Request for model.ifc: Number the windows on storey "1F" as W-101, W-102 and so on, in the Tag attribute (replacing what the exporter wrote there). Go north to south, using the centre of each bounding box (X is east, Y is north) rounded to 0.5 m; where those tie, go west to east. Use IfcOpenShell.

First a look at what the model holds.

```python
import ifcopenshell
import ifcopenshell.util.element
import ifcopenshell.util.placement

model = ifcopenshell.open("model.ifc")
print(model.schema)
storey = next(s for s in model.by_type("IfcBuildingStorey") if s.Name == "1F")
windows = [e for e in ifcopenshell.util.element.get_decomposition(storey) if e.is_a("IfcWindow")]
for e in sorted(windows, key=lambda e: e.id()):
    origin = ifcopenshell.util.placement.get_local_placement(e.ObjectPlacement)[:3, 3]
    print(e.id(), e.Tag, e.Name, origin.round(2) + 0.0, sep=" | ")
```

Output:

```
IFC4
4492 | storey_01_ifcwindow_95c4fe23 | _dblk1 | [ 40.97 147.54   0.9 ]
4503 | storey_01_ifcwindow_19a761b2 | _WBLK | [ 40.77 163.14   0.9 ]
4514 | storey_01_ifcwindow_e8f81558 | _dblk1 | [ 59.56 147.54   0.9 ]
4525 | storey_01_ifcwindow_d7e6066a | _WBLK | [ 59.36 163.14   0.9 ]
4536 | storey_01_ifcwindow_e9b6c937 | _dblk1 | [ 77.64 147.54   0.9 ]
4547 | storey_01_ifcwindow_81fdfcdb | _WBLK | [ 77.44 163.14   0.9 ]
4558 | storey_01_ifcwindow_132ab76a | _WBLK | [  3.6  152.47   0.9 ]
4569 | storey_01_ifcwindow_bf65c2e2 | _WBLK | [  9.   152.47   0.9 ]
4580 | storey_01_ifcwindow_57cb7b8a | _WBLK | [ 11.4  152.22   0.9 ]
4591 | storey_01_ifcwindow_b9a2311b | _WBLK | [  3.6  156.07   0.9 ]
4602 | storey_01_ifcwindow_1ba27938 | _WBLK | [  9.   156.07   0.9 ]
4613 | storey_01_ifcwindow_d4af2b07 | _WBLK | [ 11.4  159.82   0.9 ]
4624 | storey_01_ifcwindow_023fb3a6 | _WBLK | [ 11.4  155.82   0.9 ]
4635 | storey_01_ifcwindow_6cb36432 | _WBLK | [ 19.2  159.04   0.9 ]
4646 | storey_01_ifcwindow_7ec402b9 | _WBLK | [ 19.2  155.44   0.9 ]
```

```python
import ifcopenshell
import ifcopenshell.geom
import ifcopenshell.util.element
import ifcopenshell.util.shape

model = ifcopenshell.open("model.ifc")
settings = ifcopenshell.geom.settings()
settings.set("use-world-coords", True)


def centre(element):
    shape = ifcopenshell.geom.create_shape(settings, element)
    return ifcopenshell.util.shape.get_bbox_centroid(shape.geometry)


storey = next(s for s in model.by_type("IfcBuildingStorey") if s.Name == "1F")
windows = [e for e in ifcopenshell.util.element.get_decomposition(storey) if e.is_a("IfcWindow")]

# Insertion points can sit at a corner or the storey origin, so sort by the geometry (in metres).
centres = {e: centre(e) for e in windows}
windows.sort(key=lambda e: (-round(centres[e][1] / 0.5), centres[e][0]))

for i, e in enumerate(windows, start=1):
    number = f"W-1{i:02d}"
    e.Tag = number
    print(e.id(), number)

model.write("model_edited.ifc")
```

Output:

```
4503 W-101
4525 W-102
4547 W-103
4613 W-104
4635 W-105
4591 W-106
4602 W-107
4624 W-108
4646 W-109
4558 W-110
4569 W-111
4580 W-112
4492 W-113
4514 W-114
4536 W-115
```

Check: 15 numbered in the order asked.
